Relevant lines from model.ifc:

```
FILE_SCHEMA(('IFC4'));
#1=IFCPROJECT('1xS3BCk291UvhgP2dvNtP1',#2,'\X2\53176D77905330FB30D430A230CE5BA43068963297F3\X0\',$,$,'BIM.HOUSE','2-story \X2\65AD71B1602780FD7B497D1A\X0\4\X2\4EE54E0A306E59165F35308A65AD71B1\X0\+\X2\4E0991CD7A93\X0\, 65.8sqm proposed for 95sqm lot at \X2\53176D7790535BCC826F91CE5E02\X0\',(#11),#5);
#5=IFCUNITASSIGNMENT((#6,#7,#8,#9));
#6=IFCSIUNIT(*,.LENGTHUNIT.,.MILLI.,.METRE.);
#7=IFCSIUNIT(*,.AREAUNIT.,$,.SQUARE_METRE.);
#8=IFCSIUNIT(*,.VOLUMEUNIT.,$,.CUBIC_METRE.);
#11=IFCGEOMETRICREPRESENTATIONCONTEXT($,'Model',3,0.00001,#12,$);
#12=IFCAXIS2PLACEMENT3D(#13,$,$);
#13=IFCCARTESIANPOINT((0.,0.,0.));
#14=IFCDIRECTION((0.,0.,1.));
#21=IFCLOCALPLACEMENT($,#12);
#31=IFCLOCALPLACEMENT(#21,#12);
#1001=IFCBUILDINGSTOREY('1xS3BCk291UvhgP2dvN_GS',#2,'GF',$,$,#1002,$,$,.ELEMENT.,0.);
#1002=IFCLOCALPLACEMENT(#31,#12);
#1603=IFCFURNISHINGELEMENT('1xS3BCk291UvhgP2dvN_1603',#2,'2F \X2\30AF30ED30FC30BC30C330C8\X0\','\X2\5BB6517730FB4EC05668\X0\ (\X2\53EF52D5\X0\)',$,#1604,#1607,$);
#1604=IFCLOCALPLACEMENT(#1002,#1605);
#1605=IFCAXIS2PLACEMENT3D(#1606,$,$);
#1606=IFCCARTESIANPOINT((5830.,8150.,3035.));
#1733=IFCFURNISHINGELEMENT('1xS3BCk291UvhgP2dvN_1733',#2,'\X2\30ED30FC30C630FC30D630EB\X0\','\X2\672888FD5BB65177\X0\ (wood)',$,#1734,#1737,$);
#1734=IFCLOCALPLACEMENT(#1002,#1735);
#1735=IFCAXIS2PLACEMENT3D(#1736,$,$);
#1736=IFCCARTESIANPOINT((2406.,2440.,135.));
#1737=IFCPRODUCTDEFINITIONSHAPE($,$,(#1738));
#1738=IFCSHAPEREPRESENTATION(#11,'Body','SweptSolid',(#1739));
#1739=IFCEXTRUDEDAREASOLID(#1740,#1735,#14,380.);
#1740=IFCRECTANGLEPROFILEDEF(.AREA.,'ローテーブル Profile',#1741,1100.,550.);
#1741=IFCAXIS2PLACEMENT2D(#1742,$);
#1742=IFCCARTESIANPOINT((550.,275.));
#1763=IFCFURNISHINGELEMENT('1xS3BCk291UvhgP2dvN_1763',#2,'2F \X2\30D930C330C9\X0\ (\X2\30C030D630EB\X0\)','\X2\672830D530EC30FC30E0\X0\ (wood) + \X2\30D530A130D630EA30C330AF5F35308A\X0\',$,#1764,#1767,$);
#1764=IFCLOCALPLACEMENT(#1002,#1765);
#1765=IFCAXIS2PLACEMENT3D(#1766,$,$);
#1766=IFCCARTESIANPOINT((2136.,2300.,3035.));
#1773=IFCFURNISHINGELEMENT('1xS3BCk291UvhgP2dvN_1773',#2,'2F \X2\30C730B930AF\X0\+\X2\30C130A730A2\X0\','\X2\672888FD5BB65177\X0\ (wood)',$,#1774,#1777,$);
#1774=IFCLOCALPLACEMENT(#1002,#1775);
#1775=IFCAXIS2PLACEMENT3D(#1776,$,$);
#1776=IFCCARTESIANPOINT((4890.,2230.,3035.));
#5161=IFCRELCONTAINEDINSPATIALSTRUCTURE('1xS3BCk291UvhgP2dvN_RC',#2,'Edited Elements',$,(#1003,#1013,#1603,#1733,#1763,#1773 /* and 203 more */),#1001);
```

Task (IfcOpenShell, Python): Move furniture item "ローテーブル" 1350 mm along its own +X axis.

```python
import ifcopenshell
import ifcopenshell.api.geometry
import ifcopenshell.util.placement

model = ifcopenshell.open("model.ifc")

item = model.by_guid("1xS3BCk291UvhgP2dvN_1733")
matrix = ifcopenshell.util.placement.get_local_placement(item.ObjectPlacement)
matrix[:3, 3] += matrix[:3, 0] * 1350.0
ifcopenshell.api.geometry.edit_object_placement(model, product=item, matrix=matrix, is_si=False)

print(ifcopenshell.util.placement.get_local_placement(item.ObjectPlacement).round(3) + 0.0)

model.write("model_v2.ifc")
```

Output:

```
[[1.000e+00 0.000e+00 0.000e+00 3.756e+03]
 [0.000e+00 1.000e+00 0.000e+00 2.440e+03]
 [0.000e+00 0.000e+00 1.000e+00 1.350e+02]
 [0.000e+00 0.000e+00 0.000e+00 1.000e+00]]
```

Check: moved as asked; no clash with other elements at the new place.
